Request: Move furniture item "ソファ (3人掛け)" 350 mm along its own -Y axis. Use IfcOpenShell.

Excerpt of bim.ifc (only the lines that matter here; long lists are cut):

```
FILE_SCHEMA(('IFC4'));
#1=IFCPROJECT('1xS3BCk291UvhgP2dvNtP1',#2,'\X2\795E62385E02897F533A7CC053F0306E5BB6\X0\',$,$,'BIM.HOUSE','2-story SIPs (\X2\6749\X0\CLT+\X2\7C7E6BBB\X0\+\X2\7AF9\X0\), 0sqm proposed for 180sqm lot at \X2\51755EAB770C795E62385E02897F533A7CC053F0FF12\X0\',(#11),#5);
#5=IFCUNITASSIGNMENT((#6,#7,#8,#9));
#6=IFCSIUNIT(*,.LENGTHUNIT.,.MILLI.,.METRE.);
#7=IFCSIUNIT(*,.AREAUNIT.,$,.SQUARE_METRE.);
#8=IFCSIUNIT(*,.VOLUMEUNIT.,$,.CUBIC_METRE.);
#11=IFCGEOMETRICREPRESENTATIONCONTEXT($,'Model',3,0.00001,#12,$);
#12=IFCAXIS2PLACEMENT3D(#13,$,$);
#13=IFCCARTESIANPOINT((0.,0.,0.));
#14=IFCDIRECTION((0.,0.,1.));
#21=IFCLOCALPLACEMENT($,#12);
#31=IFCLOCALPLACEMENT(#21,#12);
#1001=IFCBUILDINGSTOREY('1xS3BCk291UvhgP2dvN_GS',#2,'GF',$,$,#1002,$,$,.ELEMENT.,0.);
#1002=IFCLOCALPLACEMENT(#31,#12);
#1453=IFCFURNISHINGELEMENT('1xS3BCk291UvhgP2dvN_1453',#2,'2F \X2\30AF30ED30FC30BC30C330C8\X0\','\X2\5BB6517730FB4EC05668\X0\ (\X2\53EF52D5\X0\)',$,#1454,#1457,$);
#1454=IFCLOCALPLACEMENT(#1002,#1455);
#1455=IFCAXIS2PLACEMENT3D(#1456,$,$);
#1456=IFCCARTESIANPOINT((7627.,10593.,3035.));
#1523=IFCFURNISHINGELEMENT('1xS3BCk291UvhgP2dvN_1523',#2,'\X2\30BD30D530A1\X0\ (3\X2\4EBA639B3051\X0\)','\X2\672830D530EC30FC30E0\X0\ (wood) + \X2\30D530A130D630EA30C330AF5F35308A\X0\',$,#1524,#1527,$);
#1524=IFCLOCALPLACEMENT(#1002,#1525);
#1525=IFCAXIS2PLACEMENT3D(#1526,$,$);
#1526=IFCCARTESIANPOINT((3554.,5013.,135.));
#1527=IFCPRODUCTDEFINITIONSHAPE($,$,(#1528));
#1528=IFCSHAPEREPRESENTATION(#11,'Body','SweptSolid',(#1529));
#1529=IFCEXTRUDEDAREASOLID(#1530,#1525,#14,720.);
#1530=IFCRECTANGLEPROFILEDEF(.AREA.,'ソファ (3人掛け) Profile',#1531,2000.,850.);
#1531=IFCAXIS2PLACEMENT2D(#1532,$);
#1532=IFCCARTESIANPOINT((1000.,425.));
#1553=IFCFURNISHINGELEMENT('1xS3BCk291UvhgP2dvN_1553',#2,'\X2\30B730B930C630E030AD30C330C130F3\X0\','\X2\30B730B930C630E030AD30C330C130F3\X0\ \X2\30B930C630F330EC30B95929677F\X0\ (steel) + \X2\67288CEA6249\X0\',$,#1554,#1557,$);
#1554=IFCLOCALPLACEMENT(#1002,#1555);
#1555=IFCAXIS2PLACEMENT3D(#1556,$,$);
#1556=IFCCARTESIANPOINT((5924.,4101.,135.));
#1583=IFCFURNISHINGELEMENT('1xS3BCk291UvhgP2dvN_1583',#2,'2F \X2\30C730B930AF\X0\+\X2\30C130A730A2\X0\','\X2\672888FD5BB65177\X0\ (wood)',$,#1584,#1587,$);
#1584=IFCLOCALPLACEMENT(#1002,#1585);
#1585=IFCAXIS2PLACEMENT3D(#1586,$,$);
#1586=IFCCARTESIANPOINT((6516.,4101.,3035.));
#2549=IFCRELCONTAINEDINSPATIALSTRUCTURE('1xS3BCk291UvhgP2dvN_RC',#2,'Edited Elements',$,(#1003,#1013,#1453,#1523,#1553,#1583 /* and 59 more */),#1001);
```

```python
import ifcopenshell
import ifcopenshell.api.geometry
import ifcopenshell.util.placement

model = ifcopenshell.open("bim.ifc")

item = model.by_guid("1xS3BCk291UvhgP2dvN_1523")
matrix = ifcopenshell.util.placement.get_local_placement(item.ObjectPlacement)
matrix[:3, 3] -= matrix[:3, 1] * 350.0
ifcopenshell.api.geometry.edit_object_placement(model, product=item, matrix=matrix, is_si=False)

print(ifcopenshell.util.placement.get_local_placement(item.ObjectPlacement).round(3) + 0.0)

model.write("bim_updated.ifc")
```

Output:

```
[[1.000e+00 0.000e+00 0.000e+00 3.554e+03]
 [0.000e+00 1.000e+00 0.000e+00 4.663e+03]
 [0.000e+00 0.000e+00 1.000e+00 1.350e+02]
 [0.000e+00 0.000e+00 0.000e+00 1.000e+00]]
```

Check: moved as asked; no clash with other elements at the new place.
